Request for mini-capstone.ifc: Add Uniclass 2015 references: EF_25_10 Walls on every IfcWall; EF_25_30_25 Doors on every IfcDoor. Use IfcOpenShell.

First a look at what the model holds.

```python
import ifcopenshell

model = ifcopenshell.open("mini-capstone.ifc")
print(model.schema)
print("classifications:", [c.Name for c in model.by_type("IfcClassification")])
for ifc_class in ("IfcDoor", "IfcRoof", "IfcStair", "IfcWall", "IfcWindow"):
    print(ifc_class, len(model.by_type(ifc_class)))
```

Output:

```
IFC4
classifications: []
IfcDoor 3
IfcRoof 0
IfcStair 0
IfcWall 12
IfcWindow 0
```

```python
import ifcopenshell
import ifcopenshell.api.classification

model = ifcopenshell.open("mini-capstone.ifc")

system = ifcopenshell.api.classification.add_classification(model, classification="Uniclass 2015")

codes = {
    "IfcWall": ("EF_25_10", "Walls"),
    "IfcDoor": ("EF_25_30_25", "Doors"),
}
for ifc_class, (code, name) in codes.items():
    products = model.by_type(ifc_class)
    ifcopenshell.api.classification.add_reference(
        model, products=products, classification=system, identification=code, name=name
    )
    print(code, len(products))

model.write("mini-capstone_rev.ifc")
```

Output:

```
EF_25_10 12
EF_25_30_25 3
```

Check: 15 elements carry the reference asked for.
